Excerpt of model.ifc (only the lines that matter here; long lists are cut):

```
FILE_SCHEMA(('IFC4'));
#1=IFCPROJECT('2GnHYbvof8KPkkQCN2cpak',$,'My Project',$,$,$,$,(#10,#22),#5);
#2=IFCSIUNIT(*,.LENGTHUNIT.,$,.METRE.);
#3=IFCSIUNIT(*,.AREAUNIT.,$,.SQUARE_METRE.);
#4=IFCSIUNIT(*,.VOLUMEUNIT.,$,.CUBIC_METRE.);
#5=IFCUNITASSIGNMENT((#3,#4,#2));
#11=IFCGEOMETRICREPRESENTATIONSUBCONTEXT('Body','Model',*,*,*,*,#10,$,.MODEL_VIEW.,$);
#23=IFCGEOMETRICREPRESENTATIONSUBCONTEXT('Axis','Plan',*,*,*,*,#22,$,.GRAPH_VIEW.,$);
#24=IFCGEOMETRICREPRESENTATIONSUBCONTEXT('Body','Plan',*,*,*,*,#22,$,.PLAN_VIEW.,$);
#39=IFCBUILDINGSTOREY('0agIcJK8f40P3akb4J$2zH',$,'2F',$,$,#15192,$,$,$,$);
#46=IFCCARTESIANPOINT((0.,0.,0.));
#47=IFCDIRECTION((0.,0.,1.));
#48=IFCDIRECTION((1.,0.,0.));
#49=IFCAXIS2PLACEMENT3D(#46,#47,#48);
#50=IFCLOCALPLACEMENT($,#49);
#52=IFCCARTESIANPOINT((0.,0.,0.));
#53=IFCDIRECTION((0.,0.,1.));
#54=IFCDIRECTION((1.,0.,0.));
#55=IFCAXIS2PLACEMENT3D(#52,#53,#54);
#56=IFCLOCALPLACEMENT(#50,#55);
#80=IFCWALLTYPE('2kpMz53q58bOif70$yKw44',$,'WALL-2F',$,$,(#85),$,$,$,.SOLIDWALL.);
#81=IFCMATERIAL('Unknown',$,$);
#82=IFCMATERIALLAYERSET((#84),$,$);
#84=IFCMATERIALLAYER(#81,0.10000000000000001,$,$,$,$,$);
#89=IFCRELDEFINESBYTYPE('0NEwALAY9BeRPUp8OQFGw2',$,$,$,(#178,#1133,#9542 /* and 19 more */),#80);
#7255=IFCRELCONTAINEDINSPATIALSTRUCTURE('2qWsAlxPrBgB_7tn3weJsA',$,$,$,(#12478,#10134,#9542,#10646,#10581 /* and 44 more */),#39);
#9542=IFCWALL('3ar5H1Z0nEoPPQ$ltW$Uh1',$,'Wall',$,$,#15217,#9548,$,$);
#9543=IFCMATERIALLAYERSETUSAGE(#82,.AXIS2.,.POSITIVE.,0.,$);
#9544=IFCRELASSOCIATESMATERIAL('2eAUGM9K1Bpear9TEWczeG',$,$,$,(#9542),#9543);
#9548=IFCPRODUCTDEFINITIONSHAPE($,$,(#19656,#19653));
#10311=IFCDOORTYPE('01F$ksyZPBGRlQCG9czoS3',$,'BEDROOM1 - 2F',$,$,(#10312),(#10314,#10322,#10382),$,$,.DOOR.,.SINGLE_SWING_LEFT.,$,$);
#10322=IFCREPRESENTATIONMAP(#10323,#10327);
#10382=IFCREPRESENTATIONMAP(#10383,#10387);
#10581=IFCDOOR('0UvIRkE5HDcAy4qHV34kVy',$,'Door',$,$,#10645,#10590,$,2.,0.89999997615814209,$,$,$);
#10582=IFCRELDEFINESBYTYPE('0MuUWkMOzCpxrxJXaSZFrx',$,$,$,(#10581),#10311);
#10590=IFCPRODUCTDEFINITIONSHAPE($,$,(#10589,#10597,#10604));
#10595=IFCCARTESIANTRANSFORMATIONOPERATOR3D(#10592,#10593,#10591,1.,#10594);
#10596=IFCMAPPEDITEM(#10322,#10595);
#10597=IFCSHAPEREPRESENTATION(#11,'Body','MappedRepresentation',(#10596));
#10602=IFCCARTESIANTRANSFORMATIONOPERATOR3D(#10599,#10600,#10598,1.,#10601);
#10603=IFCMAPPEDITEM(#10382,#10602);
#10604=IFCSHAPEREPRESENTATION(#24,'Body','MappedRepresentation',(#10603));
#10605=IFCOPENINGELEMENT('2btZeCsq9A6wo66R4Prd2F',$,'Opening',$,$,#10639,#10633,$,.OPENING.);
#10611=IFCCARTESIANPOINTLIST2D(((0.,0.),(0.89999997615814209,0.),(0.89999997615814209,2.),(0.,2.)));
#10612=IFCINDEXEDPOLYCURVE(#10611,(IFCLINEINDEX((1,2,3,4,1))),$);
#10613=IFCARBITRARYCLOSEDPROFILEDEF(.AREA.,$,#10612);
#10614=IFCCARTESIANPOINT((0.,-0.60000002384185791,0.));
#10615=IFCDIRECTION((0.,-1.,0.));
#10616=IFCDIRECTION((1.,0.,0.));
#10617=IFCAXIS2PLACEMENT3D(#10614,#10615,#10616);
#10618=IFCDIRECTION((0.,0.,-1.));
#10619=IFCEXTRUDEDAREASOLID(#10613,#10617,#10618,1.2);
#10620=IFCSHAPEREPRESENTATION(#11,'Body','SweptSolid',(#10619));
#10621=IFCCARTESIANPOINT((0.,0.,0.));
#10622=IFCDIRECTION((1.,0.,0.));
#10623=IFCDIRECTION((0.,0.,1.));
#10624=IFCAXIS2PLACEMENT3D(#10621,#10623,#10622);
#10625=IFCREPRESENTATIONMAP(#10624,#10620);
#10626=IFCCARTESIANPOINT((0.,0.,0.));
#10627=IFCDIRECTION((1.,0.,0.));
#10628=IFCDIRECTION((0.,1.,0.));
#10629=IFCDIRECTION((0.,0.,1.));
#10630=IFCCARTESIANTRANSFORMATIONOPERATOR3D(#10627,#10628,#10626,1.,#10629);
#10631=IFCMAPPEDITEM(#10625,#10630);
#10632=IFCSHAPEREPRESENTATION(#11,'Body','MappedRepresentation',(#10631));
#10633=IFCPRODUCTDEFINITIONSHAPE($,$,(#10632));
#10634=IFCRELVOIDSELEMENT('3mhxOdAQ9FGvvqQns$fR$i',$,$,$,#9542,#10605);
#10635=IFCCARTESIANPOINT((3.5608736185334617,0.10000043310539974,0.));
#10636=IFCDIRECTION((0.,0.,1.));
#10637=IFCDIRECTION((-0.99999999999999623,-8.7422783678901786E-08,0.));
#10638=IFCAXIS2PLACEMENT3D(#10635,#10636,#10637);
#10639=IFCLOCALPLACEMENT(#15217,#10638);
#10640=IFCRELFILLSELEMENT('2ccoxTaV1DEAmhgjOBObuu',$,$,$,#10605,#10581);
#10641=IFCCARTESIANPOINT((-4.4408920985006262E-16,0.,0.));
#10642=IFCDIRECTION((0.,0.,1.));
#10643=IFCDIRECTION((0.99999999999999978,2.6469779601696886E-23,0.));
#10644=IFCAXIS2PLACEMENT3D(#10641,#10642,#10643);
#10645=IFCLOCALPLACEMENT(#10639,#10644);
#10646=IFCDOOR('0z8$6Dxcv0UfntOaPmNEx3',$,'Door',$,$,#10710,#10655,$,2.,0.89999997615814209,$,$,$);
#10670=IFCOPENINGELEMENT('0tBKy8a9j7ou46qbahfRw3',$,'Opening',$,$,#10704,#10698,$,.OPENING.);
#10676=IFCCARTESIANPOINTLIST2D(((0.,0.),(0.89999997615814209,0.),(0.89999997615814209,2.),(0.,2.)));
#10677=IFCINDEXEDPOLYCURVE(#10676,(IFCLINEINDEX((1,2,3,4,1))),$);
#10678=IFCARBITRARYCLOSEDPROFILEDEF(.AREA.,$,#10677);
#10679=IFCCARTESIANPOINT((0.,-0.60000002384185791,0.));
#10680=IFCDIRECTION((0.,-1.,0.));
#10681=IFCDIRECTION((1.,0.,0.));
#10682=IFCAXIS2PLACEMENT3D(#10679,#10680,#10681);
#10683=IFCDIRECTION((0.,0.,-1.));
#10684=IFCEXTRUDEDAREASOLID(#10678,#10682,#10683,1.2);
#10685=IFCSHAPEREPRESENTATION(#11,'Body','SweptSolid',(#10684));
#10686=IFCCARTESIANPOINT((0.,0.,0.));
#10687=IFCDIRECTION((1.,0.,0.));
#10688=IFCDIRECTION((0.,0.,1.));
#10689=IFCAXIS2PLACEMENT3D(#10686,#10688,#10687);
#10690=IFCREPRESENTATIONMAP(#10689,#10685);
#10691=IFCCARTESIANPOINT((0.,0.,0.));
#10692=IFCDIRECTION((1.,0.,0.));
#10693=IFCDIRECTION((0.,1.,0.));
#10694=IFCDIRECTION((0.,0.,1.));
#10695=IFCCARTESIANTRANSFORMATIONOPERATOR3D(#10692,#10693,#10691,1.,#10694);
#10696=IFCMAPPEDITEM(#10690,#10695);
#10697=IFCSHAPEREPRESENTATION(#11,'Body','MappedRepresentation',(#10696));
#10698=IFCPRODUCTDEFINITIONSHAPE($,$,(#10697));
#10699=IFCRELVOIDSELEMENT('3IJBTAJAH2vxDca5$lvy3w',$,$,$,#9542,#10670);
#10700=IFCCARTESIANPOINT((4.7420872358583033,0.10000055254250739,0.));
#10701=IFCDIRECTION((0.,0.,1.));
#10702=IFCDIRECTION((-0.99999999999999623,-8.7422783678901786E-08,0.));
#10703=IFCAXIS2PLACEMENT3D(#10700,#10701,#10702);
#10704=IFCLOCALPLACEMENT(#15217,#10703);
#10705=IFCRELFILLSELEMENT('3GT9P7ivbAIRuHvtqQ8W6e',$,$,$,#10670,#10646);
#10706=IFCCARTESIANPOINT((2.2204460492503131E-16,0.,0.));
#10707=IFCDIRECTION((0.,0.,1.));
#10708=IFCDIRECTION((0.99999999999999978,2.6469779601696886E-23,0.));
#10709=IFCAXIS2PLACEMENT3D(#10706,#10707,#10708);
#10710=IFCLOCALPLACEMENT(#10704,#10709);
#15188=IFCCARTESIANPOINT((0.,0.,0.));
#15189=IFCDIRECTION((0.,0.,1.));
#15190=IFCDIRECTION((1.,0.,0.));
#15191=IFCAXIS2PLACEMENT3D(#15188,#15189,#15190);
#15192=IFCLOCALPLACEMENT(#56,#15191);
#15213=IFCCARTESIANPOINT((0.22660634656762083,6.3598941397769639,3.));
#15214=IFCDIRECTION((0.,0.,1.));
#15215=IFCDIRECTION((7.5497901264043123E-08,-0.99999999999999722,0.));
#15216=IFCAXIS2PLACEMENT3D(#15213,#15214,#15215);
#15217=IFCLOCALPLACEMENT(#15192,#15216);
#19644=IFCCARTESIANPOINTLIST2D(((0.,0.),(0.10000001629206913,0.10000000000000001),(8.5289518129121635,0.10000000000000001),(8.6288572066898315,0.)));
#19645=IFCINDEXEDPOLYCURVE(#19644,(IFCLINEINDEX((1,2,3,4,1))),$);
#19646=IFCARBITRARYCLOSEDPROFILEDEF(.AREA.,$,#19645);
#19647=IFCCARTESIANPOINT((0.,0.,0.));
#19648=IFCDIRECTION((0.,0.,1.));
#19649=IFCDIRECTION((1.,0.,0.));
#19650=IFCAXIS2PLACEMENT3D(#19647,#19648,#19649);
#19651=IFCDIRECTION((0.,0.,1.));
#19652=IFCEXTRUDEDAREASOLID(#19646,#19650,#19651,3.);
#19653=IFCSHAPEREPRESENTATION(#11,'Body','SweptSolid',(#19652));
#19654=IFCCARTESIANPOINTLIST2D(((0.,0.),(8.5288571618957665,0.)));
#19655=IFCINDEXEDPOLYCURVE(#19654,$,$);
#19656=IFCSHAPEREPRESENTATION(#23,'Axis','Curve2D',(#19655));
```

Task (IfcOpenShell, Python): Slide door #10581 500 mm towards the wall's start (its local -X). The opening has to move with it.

```python
import ifcopenshell
import ifcopenshell.api.geometry
import ifcopenshell.util.placement

model = ifcopenshell.open("model.ifc")

door = model.by_guid("0UvIRkE5HDcAy4qHV34kVy")
opening = door.FillsVoids[0].RelatingOpeningElement
wall = opening.VoidsElements[0].RelatingBuildingElement

wall_matrix = ifcopenshell.util.placement.get_local_placement(wall.ObjectPlacement)
shift = wall_matrix[:3, 0] * -0.5
before = ifcopenshell.util.placement.get_local_placement(door.ObjectPlacement)[:3, 3].copy()

# The door is placed relative to its opening, so it follows when the opening moves.
matrix = ifcopenshell.util.placement.get_local_placement(opening.ObjectPlacement)
matrix[:3, 3] += shift
ifcopenshell.api.geometry.edit_object_placement(
    model, product=opening, matrix=matrix, is_si=False, should_transform_children=True
)

after = ifcopenshell.util.placement.get_local_placement(door.ObjectPlacement)[:3, 3]
print("door moved by", (after - before).round(3) + 0.0)

model.write("model_rev.ifc")
```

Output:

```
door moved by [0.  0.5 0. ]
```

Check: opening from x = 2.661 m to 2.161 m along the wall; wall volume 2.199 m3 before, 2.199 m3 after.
